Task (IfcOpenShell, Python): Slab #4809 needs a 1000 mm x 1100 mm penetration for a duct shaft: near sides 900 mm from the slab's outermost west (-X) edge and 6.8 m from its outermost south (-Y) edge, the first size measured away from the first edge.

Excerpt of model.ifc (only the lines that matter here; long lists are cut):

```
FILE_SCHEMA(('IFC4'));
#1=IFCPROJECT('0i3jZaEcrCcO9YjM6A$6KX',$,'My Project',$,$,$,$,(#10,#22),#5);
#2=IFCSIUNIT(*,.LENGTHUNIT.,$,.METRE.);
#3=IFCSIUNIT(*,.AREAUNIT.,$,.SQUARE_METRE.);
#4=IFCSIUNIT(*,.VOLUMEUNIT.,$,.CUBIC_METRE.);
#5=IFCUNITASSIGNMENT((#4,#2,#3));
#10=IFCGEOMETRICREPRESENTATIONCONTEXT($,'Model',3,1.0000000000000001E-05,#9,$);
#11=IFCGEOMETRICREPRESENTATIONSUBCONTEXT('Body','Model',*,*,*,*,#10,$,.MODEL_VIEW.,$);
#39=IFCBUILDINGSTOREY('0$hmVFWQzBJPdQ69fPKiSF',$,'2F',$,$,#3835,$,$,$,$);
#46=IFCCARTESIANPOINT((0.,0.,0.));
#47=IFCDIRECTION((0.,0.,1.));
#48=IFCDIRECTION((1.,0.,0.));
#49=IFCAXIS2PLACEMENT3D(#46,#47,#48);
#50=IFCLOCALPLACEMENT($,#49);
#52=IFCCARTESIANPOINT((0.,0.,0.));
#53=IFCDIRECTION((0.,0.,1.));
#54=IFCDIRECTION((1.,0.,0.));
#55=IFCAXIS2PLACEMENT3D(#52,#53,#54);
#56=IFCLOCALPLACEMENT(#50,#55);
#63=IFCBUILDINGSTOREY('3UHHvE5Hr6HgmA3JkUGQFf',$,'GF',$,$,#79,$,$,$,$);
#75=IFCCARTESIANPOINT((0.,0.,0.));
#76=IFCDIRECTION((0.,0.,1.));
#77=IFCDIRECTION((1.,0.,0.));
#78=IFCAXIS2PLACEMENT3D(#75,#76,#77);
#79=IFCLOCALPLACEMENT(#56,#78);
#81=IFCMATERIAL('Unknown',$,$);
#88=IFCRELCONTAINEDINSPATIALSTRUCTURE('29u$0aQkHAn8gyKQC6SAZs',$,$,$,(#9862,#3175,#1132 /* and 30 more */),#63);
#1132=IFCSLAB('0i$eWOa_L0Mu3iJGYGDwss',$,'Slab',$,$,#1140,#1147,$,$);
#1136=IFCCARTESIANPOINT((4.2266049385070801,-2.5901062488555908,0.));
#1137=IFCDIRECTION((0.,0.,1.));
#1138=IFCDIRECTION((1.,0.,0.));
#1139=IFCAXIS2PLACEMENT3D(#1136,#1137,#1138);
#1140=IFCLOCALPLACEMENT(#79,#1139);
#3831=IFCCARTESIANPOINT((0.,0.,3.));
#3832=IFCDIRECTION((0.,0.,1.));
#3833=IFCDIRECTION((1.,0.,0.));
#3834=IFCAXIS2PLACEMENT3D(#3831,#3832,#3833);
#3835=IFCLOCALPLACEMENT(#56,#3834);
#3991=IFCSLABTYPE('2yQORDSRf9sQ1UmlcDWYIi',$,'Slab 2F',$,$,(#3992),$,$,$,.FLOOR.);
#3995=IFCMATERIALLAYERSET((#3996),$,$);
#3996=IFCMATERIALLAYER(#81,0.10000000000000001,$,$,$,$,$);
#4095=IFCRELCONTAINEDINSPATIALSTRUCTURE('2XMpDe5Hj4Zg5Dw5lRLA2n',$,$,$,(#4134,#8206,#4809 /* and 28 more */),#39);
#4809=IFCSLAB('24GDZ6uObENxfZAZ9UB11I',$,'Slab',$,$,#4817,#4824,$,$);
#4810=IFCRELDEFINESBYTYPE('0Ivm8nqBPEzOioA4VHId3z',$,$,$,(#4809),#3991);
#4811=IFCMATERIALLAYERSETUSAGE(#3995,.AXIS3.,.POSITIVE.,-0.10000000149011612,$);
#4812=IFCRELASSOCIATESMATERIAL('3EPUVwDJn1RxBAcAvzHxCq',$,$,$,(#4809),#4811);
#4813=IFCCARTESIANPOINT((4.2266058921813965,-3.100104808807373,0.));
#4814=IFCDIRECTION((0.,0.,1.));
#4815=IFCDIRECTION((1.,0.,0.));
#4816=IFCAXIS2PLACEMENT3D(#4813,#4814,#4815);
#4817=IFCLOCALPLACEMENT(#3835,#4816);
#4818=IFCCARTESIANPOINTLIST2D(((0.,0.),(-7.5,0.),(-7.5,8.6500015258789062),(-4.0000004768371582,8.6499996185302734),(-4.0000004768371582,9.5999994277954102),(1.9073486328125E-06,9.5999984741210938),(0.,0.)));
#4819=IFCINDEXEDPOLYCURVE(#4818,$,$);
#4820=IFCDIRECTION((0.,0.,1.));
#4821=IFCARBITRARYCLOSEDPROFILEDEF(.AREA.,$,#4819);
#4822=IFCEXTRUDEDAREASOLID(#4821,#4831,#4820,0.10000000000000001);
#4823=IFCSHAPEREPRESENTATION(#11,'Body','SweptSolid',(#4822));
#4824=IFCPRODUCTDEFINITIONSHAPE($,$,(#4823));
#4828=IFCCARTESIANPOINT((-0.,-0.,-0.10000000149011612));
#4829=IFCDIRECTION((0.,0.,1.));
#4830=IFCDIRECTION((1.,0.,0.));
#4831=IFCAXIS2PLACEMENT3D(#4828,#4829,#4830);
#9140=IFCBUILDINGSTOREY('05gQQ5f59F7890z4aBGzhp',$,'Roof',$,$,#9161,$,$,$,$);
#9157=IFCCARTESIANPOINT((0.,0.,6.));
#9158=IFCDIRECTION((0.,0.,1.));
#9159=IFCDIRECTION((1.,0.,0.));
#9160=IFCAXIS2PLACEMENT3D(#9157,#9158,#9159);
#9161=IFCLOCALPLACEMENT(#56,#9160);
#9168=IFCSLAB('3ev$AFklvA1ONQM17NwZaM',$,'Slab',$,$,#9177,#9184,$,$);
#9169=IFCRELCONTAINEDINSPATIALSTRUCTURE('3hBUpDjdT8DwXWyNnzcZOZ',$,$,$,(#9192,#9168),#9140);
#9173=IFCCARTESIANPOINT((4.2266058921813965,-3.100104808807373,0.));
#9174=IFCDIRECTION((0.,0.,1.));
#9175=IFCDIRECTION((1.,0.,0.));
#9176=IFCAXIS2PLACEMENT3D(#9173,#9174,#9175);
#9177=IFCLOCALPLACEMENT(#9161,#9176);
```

```python
import numpy as np
import ifcopenshell
import ifcopenshell.api.feature
import ifcopenshell.api.geometry
import ifcopenshell.api.root
import ifcopenshell.geom
import ifcopenshell.util.placement
import ifcopenshell.util.representation
import ifcopenshell.util.shape
import ifcopenshell.util.unit

model = ifcopenshell.open("model.ifc")
unit_scale = ifcopenshell.util.unit.calculate_unit_scale(model)
settings = ifcopenshell.geom.settings()


def volume(element):
    """Net volume in cubic metres, openings subtracted."""
    shape = ifcopenshell.geom.create_shape(settings, element)
    return ifcopenshell.util.shape.get_volume(shape.geometry)


slab = model.by_id(4809)
before = volume(slab)

# Extent in the slab's own axes, in metres. The edges named are its -X and -Y sides.
slab_shape = ifcopenshell.geom.create_shape(settings, slab)
vertices = ifcopenshell.util.shape.get_vertices(slab_shape.geometry)
x_min, y_min, bottom = vertices.min(axis=0)
top = vertices[:, 2].max()

opening = ifcopenshell.api.root.create_entity(model, ifc_class="IfcOpeningElement", name="Duct shaft opening", predefined_type="OPENING")
context = ifcopenshell.util.representation.get_context(model, "Model", "Body", "MODEL_VIEW")
width, depth = 1, 1.1
outline = [(0.0, 0.0), (width, 0.0), (width, depth), (0.0, depth), (0.0, 0.0)]
# Overshoot both faces by 50 mm so the cut is clean.
shape = ifcopenshell.api.geometry.add_slab_representation(
    model, context=context, depth=top - bottom + 0.1, polyline=outline
)
ifcopenshell.api.geometry.assign_representation(model, product=opening, representation=shape)

matrix = ifcopenshell.util.placement.get_local_placement(slab.ObjectPlacement)
matrix[:, 3] = matrix @ np.append(np.array([x_min + 0.9, y_min + 6.8, bottom - 0.05]) / unit_scale, 1.0)
ifcopenshell.api.geometry.edit_object_placement(model, product=opening, matrix=matrix, is_si=False)
ifcopenshell.api.feature.add_feature(model, feature=opening, element=slab)

after = volume(slab)

print(f"slab volume {before:.3f} -> {after:.3f} m3")

model.write("model_updated.ifc")
```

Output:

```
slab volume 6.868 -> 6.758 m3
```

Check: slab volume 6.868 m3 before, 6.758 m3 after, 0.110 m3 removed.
